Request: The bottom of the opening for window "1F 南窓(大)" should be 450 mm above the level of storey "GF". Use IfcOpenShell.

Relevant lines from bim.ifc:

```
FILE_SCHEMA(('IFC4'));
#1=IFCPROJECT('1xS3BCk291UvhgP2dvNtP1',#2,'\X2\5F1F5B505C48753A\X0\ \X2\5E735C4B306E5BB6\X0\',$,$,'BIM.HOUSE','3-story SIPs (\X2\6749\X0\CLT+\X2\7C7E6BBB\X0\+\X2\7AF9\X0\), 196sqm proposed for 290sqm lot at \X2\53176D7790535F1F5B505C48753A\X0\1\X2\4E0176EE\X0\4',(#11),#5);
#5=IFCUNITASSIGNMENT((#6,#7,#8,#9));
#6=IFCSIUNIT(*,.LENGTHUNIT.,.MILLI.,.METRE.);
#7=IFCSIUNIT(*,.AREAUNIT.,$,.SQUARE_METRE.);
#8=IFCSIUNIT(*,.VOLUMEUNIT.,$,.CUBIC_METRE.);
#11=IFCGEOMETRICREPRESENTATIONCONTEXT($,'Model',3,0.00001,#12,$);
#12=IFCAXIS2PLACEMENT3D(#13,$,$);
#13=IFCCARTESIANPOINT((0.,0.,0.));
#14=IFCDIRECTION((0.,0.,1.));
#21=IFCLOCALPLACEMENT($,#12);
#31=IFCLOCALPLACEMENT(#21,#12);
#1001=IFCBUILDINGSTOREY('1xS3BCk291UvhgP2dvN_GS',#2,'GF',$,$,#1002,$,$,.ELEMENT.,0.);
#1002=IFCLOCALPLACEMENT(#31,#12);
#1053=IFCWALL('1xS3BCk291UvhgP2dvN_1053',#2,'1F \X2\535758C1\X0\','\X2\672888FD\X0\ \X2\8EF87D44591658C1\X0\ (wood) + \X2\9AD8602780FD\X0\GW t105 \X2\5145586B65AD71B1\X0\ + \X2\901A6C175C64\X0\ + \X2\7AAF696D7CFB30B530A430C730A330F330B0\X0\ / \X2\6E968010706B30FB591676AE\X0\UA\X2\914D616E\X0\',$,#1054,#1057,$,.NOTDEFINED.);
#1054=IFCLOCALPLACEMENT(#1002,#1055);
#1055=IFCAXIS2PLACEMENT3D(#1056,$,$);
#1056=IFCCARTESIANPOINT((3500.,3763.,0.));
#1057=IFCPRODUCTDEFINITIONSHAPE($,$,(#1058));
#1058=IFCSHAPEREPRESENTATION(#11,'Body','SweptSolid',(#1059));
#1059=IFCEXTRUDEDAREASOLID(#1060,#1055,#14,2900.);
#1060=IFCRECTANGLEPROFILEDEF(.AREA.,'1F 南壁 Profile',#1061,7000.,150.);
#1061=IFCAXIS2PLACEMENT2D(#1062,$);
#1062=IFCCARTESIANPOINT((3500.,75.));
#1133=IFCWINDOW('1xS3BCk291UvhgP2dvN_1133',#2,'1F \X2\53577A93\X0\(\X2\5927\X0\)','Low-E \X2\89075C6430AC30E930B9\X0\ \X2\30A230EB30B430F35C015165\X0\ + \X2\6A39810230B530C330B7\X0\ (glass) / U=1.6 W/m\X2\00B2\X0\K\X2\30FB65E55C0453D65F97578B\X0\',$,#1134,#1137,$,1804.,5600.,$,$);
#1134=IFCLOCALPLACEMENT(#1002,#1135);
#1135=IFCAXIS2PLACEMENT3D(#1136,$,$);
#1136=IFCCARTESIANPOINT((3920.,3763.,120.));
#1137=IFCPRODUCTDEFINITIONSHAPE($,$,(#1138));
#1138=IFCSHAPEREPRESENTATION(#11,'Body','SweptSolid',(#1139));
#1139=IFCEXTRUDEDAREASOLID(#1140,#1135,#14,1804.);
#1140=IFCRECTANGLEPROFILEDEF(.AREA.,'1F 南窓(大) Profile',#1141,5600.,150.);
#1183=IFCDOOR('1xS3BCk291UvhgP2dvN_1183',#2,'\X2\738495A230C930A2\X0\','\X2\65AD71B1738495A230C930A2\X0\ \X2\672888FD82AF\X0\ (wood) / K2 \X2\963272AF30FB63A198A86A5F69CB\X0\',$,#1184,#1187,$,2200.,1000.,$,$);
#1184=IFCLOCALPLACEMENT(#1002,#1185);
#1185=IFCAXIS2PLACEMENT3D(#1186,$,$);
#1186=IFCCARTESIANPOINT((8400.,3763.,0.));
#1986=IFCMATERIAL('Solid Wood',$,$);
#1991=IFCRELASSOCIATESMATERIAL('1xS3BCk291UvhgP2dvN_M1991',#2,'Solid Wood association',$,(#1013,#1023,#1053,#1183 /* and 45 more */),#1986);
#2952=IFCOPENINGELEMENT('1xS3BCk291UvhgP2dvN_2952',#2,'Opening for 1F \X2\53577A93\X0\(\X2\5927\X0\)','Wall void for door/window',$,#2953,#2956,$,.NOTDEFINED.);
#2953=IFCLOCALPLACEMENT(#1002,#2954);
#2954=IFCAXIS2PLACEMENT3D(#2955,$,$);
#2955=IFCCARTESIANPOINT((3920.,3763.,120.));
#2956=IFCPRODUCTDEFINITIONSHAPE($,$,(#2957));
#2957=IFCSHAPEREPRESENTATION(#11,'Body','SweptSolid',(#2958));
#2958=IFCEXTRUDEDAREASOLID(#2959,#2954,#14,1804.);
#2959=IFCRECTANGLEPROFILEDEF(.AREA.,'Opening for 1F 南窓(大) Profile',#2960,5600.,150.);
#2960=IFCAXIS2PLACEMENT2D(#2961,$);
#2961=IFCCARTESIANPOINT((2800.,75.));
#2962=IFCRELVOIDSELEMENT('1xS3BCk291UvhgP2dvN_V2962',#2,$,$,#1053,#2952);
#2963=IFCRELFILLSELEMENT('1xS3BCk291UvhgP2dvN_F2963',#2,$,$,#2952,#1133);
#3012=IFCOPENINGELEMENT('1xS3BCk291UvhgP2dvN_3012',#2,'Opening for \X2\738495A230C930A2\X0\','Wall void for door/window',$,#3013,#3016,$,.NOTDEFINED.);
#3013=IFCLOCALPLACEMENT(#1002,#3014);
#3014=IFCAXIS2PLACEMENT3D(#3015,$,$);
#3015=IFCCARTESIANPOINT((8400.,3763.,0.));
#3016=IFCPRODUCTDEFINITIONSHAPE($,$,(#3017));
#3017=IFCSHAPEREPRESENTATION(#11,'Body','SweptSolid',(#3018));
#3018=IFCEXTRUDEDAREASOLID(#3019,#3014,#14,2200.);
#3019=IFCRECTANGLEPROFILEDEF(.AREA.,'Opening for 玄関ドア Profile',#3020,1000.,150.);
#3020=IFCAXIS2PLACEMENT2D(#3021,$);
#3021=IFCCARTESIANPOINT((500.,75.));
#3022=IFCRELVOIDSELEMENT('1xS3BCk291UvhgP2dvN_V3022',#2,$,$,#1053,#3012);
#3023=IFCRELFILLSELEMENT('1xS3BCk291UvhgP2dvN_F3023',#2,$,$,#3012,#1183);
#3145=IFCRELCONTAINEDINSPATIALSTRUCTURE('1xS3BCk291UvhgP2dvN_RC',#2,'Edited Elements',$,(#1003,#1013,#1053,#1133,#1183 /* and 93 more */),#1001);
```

```python
import numpy as np
import ifcopenshell
import ifcopenshell.api.geometry
import ifcopenshell.geom
import ifcopenshell.util.element
import ifcopenshell.util.placement
import ifcopenshell.util.shape
import ifcopenshell.util.unit

model = ifcopenshell.open("bim.ifc")
unit_scale = ifcopenshell.util.unit.calculate_unit_scale(model)

window = model.by_guid("1xS3BCk291UvhgP2dvN_1133")
opening = window.FillsVoids[0].RelatingOpeningElement
storey = ifcopenshell.util.element.get_container(window, ifc_class="IfcBuildingStorey")
level = ifcopenshell.util.placement.get_local_placement(storey.ObjectPlacement)[2, 3]

# The opening's origin need not be at the sill, so measure its lowest point.
shape = ifcopenshell.geom.create_shape(ifcopenshell.geom.settings(), opening)
bottom = ifcopenshell.util.shape.get_shape_bottom_elevation(shape, shape.geometry) / unit_scale
dz = level + 0.45 / unit_scale - bottom

shift = np.array([0.0, 0.0, dz])
# The window is not placed relative to its opening, so move both.
for product in (opening, window):
    matrix = ifcopenshell.util.placement.get_local_placement(product.ObjectPlacement)
    matrix[:3, 3] += shift
    ifcopenshell.api.geometry.edit_object_placement(model, product=product, matrix=matrix, is_si=False)

print(f"moved by {dz * unit_scale:+.3f} m")

model.write("bim_edited.ifc")
```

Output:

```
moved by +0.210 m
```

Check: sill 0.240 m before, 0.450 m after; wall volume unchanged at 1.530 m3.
